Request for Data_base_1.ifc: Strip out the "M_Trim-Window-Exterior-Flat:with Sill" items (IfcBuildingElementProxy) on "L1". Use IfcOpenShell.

First a look at what the model holds.

```python
import ifcopenshell
import ifcopenshell.util.element

model = ifcopenshell.open("Data_base_1.ifc")
print(model.schema)
storey = next(s for s in model.by_type("IfcBuildingStorey") if s.Name == "L1")
proxies = [e for e in ifcopenshell.util.element.get_decomposition(storey) if e.is_a("IfcBuildingElementProxy")]
seen = {}
for e in proxies:
    element_type = ifcopenshell.util.element.get_type(e)
    name = element_type.Name if element_type not in (None, e) else None
    seen[name] = seen.get(name, 0) + 1
for name, count in sorted(seen.items(), key=str):
    print(count, "x", name)
```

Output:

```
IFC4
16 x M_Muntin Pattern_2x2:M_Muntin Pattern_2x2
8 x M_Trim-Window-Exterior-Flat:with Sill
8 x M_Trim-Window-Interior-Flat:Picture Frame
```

```python
import ifcopenshell
import ifcopenshell.api.root
import ifcopenshell.util.element

model = ifcopenshell.open("Data_base_1.ifc")

storey = next(s for s in model.by_type("IfcBuildingStorey") if s.Name == "L1")
proxies = [e for e in ifcopenshell.util.element.get_decomposition(storey) if e.is_a("IfcBuildingElementProxy")]
targets = [e for e in proxies if (t := ifcopenshell.util.element.get_type(e)) not in (None, e) and t.Name == "M_Trim-Window-Exterior-Flat:with Sill"]

for e in targets:
    ifcopenshell.api.root.remove_product(model, product=e)
print(len(targets), "removed")

model.write("Data_base_1_edited.ifc")
```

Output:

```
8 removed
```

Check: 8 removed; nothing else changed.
